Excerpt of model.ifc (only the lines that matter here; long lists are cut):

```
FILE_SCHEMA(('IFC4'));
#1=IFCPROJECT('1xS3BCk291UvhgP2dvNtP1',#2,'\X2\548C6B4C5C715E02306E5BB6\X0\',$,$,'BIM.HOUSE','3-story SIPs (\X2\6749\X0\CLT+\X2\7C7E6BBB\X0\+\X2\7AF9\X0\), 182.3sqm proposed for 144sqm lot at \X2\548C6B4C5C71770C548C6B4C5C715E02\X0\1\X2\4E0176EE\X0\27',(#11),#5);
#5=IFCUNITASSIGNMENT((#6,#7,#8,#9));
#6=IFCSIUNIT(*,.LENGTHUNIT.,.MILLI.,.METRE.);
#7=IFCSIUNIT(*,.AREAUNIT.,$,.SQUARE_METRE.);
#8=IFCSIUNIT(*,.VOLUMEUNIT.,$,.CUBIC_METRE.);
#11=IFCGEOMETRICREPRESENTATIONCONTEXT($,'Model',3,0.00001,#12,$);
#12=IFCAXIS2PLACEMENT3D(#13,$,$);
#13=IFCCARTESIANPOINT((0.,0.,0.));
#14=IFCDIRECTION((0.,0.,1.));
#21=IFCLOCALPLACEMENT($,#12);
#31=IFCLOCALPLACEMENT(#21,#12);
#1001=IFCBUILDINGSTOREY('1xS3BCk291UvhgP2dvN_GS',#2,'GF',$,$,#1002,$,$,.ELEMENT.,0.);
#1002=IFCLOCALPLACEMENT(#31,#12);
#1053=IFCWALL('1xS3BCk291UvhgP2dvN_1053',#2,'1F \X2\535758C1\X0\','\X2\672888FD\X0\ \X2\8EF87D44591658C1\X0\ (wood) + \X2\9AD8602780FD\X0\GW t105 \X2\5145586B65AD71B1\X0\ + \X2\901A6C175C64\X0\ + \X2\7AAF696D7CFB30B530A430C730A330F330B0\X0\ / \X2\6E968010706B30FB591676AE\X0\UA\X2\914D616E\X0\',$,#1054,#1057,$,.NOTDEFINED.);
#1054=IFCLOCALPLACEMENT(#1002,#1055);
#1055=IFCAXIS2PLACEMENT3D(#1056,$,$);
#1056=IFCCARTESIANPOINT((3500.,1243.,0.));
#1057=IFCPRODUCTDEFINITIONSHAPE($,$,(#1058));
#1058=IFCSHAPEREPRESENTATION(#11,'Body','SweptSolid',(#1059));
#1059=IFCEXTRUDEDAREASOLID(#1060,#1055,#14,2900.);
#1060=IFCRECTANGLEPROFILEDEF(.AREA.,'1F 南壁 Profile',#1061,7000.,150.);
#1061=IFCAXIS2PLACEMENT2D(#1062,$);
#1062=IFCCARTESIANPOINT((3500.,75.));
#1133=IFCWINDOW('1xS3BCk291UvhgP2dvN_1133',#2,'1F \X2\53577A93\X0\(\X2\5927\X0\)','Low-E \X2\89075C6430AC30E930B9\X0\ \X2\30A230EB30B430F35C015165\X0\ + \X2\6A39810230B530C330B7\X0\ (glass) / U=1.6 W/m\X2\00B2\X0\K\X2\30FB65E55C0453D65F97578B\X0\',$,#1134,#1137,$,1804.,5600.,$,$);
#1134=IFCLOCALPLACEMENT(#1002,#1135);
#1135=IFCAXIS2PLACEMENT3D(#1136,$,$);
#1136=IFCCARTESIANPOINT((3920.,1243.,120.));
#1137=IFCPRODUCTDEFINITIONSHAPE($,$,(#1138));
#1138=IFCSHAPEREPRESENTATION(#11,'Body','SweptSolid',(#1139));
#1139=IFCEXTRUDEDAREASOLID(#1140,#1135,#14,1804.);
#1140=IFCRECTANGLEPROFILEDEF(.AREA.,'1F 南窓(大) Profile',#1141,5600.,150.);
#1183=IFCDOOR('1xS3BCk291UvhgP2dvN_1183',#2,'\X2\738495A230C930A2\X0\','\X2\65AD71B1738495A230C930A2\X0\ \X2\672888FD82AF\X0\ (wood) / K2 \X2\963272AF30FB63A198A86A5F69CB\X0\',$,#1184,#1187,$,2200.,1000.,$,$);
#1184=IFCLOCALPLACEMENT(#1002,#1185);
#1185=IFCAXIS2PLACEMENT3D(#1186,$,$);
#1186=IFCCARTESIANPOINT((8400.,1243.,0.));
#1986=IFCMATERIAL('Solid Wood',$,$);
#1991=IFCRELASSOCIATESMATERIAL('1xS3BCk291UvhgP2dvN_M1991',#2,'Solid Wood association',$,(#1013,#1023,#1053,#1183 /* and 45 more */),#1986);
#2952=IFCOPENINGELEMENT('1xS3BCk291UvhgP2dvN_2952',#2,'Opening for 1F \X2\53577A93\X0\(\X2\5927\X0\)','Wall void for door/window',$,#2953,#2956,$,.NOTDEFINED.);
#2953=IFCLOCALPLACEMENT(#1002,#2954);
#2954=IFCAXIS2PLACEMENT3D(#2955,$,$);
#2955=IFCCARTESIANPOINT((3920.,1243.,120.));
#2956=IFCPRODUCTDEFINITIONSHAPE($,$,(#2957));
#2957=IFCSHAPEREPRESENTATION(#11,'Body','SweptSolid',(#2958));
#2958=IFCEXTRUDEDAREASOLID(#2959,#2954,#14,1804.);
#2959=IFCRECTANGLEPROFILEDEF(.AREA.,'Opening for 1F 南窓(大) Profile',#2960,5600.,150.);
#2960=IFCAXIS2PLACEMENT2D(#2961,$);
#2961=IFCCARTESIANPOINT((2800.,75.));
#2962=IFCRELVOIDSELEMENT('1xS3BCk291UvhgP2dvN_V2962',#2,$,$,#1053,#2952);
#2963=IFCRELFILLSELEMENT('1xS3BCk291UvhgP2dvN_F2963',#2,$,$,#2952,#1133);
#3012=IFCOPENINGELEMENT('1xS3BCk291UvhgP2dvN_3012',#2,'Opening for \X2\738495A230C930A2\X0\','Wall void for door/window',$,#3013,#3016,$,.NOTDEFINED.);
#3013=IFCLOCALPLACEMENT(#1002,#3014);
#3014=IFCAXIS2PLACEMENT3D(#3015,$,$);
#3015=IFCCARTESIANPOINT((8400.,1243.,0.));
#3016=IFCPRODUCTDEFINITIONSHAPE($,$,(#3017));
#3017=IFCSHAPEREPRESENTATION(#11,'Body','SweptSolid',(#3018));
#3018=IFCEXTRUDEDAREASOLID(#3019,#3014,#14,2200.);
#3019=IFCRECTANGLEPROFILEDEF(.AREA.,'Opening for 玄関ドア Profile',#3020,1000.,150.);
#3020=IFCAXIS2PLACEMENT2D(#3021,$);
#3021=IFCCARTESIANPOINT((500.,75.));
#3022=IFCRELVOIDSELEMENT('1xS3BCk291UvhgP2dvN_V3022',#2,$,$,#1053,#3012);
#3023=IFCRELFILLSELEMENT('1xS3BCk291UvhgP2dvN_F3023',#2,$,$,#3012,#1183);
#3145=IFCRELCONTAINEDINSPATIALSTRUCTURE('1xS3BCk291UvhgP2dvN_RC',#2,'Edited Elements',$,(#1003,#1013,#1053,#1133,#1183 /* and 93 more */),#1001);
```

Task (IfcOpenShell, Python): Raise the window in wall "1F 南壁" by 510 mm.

```python
import numpy as np
import ifcopenshell
import ifcopenshell.api.geometry
import ifcopenshell.util.placement
import ifcopenshell.util.unit

model = ifcopenshell.open("model.ifc")
unit_scale = ifcopenshell.util.unit.calculate_unit_scale(model)

window = model.by_id(1133)
opening = window.FillsVoids[0].RelatingOpeningElement
dz = 0.51 / unit_scale

shift = np.array([0.0, 0.0, dz])
# The window is not placed relative to its opening, so move both.
for product in (opening, window):
    matrix = ifcopenshell.util.placement.get_local_placement(product.ObjectPlacement)
    matrix[:3, 3] += shift
    ifcopenshell.api.geometry.edit_object_placement(model, product=product, matrix=matrix, is_si=False)

print(f"moved by {dz * unit_scale:+.3f} m")

model.write("model-out.ifc")
```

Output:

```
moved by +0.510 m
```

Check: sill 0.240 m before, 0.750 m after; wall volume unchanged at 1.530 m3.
